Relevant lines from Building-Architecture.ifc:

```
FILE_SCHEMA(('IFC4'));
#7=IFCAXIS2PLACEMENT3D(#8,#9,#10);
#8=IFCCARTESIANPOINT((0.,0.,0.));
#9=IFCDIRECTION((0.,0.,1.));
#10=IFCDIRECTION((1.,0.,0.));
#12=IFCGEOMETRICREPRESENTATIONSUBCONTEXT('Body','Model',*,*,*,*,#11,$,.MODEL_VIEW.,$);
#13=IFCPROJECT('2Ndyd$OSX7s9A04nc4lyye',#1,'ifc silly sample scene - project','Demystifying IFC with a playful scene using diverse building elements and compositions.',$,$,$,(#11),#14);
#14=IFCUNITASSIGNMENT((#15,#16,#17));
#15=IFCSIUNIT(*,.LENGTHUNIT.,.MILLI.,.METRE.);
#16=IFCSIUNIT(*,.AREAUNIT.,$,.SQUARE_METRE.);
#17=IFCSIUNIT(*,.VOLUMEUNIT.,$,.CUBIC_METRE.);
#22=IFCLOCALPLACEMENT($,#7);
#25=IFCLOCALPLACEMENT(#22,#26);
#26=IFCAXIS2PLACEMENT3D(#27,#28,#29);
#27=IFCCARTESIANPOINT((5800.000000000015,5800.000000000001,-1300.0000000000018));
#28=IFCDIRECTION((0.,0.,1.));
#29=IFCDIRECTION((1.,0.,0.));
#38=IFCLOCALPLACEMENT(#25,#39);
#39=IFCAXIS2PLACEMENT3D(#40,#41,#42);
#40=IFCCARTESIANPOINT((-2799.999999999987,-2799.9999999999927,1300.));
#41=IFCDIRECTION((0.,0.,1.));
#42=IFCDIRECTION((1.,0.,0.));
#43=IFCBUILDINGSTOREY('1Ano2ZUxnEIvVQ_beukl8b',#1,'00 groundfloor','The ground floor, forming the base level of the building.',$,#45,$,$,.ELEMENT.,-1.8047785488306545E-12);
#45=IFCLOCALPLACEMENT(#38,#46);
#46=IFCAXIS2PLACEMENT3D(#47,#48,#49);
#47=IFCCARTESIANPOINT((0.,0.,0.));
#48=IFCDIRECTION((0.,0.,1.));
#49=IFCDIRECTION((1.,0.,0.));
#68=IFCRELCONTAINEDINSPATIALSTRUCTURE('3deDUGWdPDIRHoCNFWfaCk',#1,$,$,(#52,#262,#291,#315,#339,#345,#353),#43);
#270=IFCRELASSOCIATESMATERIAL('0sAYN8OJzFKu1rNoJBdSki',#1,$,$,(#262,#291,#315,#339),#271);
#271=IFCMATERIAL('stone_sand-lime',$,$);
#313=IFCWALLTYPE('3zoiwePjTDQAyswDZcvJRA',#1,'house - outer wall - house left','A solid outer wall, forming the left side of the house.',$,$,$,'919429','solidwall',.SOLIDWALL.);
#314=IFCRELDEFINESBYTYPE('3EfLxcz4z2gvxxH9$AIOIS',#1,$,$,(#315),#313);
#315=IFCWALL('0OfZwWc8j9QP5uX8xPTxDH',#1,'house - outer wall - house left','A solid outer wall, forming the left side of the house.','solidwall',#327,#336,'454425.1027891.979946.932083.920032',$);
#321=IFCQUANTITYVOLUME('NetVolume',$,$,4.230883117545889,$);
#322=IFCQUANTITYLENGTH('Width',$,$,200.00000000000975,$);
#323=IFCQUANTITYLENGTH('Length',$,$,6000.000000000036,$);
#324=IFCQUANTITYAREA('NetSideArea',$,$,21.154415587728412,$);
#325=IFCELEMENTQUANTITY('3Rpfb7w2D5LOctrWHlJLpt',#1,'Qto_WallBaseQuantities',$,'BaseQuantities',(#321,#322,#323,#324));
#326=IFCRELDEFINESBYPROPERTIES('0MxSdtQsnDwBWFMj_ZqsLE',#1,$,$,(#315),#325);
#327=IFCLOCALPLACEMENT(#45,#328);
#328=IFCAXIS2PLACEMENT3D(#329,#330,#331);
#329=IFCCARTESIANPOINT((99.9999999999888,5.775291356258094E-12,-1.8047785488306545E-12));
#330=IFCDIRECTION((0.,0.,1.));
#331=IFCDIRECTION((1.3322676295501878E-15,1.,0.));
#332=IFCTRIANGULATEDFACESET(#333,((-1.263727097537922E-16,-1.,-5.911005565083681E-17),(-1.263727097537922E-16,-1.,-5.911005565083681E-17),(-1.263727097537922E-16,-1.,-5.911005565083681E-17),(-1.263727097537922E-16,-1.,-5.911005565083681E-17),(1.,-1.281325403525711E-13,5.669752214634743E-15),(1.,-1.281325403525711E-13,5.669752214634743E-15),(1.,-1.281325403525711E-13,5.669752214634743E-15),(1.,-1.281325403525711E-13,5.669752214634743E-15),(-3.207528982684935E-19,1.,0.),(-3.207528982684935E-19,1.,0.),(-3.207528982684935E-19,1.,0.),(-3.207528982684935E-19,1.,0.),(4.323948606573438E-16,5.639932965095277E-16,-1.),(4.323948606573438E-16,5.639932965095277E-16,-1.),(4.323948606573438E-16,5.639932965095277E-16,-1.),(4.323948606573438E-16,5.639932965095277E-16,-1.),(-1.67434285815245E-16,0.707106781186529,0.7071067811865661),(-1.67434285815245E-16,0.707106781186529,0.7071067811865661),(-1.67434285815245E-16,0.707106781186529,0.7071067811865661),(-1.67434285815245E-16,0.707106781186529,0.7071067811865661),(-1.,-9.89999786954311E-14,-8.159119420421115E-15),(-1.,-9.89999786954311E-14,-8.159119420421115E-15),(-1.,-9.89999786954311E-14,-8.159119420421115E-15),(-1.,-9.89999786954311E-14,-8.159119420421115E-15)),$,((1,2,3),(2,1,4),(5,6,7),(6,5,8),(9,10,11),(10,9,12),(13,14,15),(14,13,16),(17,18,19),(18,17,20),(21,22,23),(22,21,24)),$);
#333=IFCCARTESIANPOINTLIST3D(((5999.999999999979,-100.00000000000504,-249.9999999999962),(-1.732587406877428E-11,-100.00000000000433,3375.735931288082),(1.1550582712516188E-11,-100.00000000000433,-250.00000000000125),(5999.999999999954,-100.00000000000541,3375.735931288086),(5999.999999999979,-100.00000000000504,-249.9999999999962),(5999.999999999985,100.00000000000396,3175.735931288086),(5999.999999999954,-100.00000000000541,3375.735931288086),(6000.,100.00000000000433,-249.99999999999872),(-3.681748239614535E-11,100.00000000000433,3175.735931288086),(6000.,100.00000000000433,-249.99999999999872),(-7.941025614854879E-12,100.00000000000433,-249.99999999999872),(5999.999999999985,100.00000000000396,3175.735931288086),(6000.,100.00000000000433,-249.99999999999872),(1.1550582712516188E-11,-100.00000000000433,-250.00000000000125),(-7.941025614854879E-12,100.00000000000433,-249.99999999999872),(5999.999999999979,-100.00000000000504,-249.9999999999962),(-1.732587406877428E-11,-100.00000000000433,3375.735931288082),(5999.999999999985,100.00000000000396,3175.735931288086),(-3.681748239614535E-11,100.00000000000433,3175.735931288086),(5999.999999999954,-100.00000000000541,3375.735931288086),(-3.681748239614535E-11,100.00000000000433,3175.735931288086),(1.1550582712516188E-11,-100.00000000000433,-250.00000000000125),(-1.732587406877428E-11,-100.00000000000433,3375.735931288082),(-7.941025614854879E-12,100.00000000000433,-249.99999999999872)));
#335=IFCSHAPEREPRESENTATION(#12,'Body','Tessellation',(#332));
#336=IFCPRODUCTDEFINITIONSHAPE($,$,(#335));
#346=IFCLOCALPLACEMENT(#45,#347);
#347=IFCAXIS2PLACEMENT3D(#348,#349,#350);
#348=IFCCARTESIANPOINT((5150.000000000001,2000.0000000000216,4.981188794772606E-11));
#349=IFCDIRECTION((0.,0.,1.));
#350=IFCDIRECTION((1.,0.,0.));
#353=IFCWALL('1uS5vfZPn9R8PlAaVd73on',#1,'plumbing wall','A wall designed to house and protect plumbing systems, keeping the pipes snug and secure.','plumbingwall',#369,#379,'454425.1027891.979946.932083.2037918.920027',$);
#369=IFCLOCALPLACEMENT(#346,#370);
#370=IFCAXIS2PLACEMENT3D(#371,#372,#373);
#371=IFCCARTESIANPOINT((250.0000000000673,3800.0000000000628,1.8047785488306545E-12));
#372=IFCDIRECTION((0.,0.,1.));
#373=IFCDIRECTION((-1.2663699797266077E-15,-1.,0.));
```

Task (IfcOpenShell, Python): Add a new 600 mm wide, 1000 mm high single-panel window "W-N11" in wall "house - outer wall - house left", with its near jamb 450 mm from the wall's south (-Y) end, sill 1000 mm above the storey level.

```python
import numpy as np
import ifcopenshell
import ifcopenshell.api.feature
import ifcopenshell.api.geometry
import ifcopenshell.api.pset
import ifcopenshell.api.root
import ifcopenshell.api.spatial
import ifcopenshell.geom
import ifcopenshell.util.element
import ifcopenshell.util.placement
import ifcopenshell.util.representation
import ifcopenshell.util.shape
import ifcopenshell.util.unit

model = ifcopenshell.open("Building-Architecture.ifc")
unit_scale = ifcopenshell.util.unit.calculate_unit_scale(model)
area_scale = ifcopenshell.util.unit.calculate_unit_scale(model, "AREAUNIT")
volume_scale = ifcopenshell.util.unit.calculate_unit_scale(model, "VOLUMEUNIT")
settings = ifcopenshell.geom.settings()


def volume(element):
    """Net volume in cubic metres, openings subtracted."""
    shape = ifcopenshell.geom.create_shape(settings, element)
    return ifcopenshell.util.shape.get_volume(shape.geometry)


wall = model.by_id(315)
storey = ifcopenshell.util.element.get_container(wall, ifc_class="IfcBuildingStorey")
context = ifcopenshell.util.representation.get_context(model, "Model", "Body", "MODEL_VIEW")
before = volume(wall)

width, height, from_end, sill = 0.6, 1, 0.45, 1  # metres

# The wall runs along its own X axis, and the end named is its -X end.
wall_shape = ifcopenshell.geom.create_shape(settings, wall)
x, y, z = ifcopenshell.util.shape.get_vertices(wall_shape.geometry).T
start = x.min() + from_end
face, thickness = float(y.min()), float(y.max() - y.min())
wall_matrix = ifcopenshell.util.placement.get_local_placement(wall.ObjectPlacement)
level = ifcopenshell.util.placement.get_local_placement(storey.ObjectPlacement)[2, 3]


def in_wall(x, y):
    """Placement at x, y metres in the wall's axes, at sill height."""
    matrix = wall_matrix.copy()
    matrix[:, 3] = wall_matrix @ np.array([x / unit_scale, y / unit_scale, 0.0, 1.0])
    matrix[2, 3] = level + sill / unit_scale
    return matrix


# Opening: a box that overshoots both wall faces by 50 mm.
opening = ifcopenshell.api.root.create_entity(model, ifc_class="IfcOpeningElement", predefined_type="OPENING")
box = ifcopenshell.api.geometry.add_wall_representation(
    model, context=context, length=width, height=height, thickness=thickness + 0.1
)
ifcopenshell.api.geometry.assign_representation(model, product=opening, representation=box)
ifcopenshell.api.geometry.edit_object_placement(model, product=opening, matrix=in_wall(start, face - 0.05), is_si=False)
ifcopenshell.api.feature.add_feature(model, feature=opening, element=wall)

window = ifcopenshell.api.root.create_entity(model, ifc_class="IfcWindow", name="W-N11", predefined_type="WINDOW")
window.OverallWidth, window.OverallHeight = width / unit_scale, height / unit_scale
window.PartitioningType = "SINGLE_PANEL"
body = ifcopenshell.api.geometry.add_window_representation(
    model,
    context=context,
    overall_width=window.OverallWidth,
    overall_height=window.OverallHeight,
    partition_type="SINGLE_PANEL",
)
ifcopenshell.api.geometry.assign_representation(model, product=window, representation=body)
ifcopenshell.api.spatial.assign_container(model, products=[window], relating_structure=storey)
ifcopenshell.api.feature.add_filling(model, opening=opening, element=window)

# Centre the window in the wall's thickness.
ifcopenshell.api.geometry.edit_object_placement(model, product=window, matrix=in_wall(start, face), is_si=False)
window_shape = ifcopenshell.geom.create_shape(settings, window)
depth = ifcopenshell.util.shape.get_vertices(window_shape.geometry)[:, 1]
offset = face + thickness / 2 - (depth.min() + depth.max()) / 2
ifcopenshell.api.geometry.edit_object_placement(model, product=window, matrix=in_wall(start, offset), is_si=False)

after = volume(wall)

# Update the wall's stored quantities.
qto = model.by_id(ifcopenshell.util.element.get_pset(wall, "Qto_WallBaseQuantities", should_inherit=False)["id"])
ifcopenshell.api.pset.edit_qto(model, qto=qto, properties={
    "NetVolume": after / volume_scale,
    "NetSideArea": after / thickness / area_scale,
})

print(f"wall volume {before:.3f} -> {after:.3f} m3")

model.write("Building-Architecture-out.ifc")
```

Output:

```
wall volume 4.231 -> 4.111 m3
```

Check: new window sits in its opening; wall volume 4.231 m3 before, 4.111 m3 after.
